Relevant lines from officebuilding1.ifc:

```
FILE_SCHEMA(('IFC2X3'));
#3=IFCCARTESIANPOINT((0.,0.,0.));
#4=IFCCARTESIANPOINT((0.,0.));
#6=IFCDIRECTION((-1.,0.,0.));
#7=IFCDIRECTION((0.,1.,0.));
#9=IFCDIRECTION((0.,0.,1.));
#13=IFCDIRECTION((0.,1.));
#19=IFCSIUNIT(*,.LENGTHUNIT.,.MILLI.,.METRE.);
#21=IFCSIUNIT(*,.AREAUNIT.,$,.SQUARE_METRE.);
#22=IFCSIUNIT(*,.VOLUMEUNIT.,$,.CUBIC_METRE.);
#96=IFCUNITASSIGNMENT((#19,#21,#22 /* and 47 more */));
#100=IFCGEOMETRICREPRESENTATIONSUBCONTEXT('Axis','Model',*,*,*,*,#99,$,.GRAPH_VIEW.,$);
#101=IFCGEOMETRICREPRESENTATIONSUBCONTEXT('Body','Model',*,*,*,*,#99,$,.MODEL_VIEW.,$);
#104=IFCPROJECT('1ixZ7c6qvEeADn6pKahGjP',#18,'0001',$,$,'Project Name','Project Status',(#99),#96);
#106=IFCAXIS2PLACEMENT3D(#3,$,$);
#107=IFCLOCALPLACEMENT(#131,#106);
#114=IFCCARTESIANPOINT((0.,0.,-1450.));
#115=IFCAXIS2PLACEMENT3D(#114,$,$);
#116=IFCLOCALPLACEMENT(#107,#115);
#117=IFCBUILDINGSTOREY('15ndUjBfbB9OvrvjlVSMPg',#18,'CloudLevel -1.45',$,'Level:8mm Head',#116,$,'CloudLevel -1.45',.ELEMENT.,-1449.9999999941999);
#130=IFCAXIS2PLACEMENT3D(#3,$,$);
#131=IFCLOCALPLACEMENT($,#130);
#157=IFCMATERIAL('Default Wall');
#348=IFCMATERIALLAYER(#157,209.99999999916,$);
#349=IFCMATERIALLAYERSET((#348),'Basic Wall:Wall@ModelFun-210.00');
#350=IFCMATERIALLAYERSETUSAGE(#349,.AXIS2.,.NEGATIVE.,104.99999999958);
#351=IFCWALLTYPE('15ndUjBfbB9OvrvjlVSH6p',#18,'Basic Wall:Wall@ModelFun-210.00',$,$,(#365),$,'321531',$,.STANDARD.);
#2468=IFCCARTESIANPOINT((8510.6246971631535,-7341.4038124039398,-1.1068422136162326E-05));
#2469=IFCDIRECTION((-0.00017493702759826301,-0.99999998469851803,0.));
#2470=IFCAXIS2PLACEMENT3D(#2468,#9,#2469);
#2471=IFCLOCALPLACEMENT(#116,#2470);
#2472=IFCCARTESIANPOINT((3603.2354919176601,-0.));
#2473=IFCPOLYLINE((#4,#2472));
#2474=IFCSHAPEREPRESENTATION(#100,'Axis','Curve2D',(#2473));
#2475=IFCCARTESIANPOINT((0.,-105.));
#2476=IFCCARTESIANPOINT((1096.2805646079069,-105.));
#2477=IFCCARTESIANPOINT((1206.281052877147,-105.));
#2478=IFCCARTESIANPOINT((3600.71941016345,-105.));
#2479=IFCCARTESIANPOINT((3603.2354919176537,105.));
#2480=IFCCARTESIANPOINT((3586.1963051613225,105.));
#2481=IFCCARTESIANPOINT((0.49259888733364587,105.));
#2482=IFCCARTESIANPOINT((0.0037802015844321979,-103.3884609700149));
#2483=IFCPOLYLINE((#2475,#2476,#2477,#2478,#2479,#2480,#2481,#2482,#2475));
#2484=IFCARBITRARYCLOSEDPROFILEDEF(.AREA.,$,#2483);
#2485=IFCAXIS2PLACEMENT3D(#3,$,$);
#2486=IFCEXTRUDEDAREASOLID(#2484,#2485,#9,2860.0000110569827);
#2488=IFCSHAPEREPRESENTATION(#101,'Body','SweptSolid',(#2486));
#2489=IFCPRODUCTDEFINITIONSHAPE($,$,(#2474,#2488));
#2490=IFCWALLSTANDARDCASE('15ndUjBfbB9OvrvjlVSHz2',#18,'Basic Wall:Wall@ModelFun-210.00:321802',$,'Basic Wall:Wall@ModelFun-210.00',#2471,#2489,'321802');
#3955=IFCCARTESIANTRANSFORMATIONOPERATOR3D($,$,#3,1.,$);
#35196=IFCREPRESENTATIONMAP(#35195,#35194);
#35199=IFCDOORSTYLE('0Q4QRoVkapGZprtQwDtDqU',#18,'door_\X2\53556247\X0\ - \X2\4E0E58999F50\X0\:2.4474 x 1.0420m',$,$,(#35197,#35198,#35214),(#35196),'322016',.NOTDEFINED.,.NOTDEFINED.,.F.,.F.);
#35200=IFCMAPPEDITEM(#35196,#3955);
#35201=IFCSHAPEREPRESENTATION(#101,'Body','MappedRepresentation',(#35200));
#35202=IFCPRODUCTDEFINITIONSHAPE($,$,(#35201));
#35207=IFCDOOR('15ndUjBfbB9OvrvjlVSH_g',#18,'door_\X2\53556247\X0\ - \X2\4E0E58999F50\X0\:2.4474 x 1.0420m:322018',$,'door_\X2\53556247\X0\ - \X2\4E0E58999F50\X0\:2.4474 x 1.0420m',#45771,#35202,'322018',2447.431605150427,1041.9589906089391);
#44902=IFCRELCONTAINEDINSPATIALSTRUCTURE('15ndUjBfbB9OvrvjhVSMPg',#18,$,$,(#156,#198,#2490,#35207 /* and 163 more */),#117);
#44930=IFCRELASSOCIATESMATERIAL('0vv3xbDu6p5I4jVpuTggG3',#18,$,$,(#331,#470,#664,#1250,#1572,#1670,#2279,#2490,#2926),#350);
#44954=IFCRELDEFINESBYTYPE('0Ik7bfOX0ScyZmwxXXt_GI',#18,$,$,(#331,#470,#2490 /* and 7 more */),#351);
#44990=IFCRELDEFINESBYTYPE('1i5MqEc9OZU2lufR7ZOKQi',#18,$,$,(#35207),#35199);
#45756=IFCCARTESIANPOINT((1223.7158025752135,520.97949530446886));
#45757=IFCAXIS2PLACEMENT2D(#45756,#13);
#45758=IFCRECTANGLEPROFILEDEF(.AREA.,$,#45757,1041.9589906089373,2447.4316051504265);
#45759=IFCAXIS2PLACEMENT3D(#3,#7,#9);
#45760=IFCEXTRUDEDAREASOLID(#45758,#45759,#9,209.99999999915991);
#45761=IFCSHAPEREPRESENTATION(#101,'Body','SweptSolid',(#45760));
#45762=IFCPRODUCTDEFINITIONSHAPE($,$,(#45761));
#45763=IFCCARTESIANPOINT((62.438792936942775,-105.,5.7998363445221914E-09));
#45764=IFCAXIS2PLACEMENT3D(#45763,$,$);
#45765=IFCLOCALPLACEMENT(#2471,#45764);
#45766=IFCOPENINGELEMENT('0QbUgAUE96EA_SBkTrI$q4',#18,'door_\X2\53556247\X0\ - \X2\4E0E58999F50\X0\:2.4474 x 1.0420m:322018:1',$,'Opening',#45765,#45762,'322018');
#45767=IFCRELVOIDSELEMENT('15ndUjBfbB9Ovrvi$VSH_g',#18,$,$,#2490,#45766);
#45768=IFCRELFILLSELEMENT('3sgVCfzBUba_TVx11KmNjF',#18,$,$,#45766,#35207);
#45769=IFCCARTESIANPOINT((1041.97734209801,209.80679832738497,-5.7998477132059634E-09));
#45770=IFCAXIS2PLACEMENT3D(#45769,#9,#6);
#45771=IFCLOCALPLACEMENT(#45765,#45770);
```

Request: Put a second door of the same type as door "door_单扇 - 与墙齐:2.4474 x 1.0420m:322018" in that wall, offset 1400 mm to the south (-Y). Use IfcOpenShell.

```python
import ifcopenshell
import ifcopenshell.api.feature
import ifcopenshell.api.geometry
import ifcopenshell.api.root
import ifcopenshell.geom
import ifcopenshell.util.element
import ifcopenshell.util.placement
import ifcopenshell.util.shape

model = ifcopenshell.open("officebuilding1.ifc")
settings = ifcopenshell.geom.settings()


def volume(element):
    """Net volume in cubic metres, openings subtracted."""
    shape = ifcopenshell.geom.create_shape(settings, element)
    return ifcopenshell.util.shape.get_volume(shape.geometry)


def reuse_history(source, copy):
    """copy_class also copies each property set's owner history, people and application; keep the originals."""
    for rel in copy.IsDefinedBy:
        if rel.is_a("IfcRelDefinesByProperties") and (history := rel.RelatingPropertyDefinition.OwnerHistory):
            rel.RelatingPropertyDefinition.OwnerHistory = source.OwnerHistory
            ifcopenshell.util.element.remove_deep2(model, history)


door = model.by_guid("15ndUjBfbB9OvrvjlVSH_g")
opening = door.FillsVoids[0].RelatingOpeningElement
wall = opening.VoidsElements[0].RelatingBuildingElement
before = volume(wall)
shift = ifcopenshell.util.placement.get_local_placement(wall.ObjectPlacement)[:3, 0] * 1400.0

# copy_class copies the void relationship, type, container and properties, but no geometry.
new_opening = ifcopenshell.api.root.copy_class(model, product=opening)
new_opening.Representation = ifcopenshell.util.element.copy_deep(
    model, opening.Representation, exclude=["IfcGeometricRepresentationContext", "IfcRepresentationMap"]
)
new_opening.Name = "door_单扇 - 与墙齐:2.4474 x 1.0420m"
new_opening.Tag = None
new_door = ifcopenshell.api.root.copy_class(model, product=door)
new_door.Representation = ifcopenshell.util.element.copy_deep(
    model, door.Representation, exclude=["IfcGeometricRepresentationContext", "IfcRepresentationMap"]
)
new_door.Name = "door_单扇 - 与墙齐:2.4474 x 1.0420m"
new_door.Tag = None
reuse_history(door, new_door)
fills = ifcopenshell.api.feature.add_filling(model, opening=new_opening, element=new_door)
fills.OwnerHistory = new_door.OwnerHistory  # required in IFC2X3

for old, new in ((opening, new_opening), (door, new_door)):
    matrix = ifcopenshell.util.placement.get_local_placement(old.ObjectPlacement)
    matrix[:3, 3] += shift
    ifcopenshell.api.geometry.edit_object_placement(model, product=new, matrix=matrix, is_si=False)

after = volume(wall)

print(f"wall volume {before:.3f} -> {after:.3f} m3")

model.write("officebuilding1_v2.ifc")
```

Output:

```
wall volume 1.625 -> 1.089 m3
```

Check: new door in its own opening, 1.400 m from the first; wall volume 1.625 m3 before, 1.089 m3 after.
